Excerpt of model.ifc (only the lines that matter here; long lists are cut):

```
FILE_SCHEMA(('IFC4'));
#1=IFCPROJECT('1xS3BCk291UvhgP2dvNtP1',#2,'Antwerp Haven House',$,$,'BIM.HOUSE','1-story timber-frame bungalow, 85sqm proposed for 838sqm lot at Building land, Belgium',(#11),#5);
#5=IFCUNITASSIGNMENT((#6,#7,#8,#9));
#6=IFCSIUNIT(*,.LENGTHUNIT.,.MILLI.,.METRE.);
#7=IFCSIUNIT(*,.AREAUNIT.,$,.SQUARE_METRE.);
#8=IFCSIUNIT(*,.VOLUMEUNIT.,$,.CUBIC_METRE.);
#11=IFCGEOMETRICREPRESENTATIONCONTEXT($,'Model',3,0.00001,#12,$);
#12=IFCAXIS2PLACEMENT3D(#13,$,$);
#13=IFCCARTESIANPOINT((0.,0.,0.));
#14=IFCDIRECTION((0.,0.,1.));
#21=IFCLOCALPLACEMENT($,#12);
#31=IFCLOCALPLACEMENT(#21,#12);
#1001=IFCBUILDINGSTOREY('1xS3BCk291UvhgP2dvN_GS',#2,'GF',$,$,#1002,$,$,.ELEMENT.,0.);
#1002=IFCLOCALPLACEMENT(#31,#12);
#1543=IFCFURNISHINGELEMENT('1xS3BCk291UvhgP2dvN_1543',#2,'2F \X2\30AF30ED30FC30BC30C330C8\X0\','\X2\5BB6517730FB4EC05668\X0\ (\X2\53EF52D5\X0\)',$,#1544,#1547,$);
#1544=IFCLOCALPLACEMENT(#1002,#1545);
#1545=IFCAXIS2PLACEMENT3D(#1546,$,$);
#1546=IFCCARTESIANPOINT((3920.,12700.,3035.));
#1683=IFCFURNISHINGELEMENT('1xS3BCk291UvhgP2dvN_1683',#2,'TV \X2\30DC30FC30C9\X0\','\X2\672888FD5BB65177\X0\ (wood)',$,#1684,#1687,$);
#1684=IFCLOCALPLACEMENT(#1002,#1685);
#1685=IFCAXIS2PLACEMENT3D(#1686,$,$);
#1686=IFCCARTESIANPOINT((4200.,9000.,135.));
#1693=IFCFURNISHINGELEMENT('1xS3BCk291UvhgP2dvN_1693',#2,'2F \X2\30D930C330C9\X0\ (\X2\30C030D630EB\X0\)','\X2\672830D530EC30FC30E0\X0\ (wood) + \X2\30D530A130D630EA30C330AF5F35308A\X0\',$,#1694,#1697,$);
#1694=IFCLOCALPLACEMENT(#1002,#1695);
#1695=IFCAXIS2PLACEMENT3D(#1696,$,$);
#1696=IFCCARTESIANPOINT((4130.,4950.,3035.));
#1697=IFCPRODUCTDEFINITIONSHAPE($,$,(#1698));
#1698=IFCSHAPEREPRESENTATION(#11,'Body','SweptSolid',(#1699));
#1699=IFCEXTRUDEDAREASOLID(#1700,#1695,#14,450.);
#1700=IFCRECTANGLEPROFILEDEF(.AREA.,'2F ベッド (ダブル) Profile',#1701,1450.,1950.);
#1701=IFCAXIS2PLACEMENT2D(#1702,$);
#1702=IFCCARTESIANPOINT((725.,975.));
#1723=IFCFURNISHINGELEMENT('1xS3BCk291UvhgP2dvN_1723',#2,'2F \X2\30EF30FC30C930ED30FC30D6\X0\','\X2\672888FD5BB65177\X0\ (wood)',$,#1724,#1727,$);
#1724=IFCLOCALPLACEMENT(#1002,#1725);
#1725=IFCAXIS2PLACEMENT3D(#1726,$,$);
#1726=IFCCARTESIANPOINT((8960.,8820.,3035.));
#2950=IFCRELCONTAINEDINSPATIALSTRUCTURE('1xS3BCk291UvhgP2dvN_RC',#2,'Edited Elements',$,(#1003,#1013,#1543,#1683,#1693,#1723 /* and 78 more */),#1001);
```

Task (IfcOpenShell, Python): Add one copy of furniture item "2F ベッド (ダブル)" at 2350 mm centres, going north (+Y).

```python
import numpy as np
import ifcopenshell
import ifcopenshell.api.geometry
import ifcopenshell.api.root
import ifcopenshell.util.element
import ifcopenshell.util.placement
import ifcopenshell.util.unit

model = ifcopenshell.open("model.ifc")
unit_scale = ifcopenshell.util.unit.calculate_unit_scale(model)


def reuse_history(source, copy):
    """copy_class also copies each property set's owner history, people and application; keep the originals."""
    for rel in copy.IsDefinedBy:
        if rel.is_a("IfcRelDefinesByProperties") and (history := rel.RelatingPropertyDefinition.OwnerHistory):
            rel.RelatingPropertyDefinition.OwnerHistory = source.OwnerHistory
            ifcopenshell.util.element.remove_deep2(model, history)


source = model.by_id(1693)
base = ifcopenshell.util.placement.get_local_placement(source.ObjectPlacement)
step = np.array([0.0, 1.0, 0.0]) * 2.35 / unit_scale

for i in range(1, 2):
    copy = ifcopenshell.api.root.copy_class(model, product=source)
    copy.Representation = ifcopenshell.util.element.copy_deep(
        model, source.Representation, exclude=["IfcGeometricRepresentationContext", "IfcRepresentationMap"]
    )
    reuse_history(source, copy)
    matrix = base.copy()
    matrix[:3, 3] += i * step
    print("added at", matrix[:3, 3].round(3) + 0.0)
    ifcopenshell.api.geometry.edit_object_placement(model, product=copy, matrix=matrix, is_si=False)

model.write("model_edited.ifc")
```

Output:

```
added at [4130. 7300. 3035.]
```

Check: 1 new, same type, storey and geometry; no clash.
